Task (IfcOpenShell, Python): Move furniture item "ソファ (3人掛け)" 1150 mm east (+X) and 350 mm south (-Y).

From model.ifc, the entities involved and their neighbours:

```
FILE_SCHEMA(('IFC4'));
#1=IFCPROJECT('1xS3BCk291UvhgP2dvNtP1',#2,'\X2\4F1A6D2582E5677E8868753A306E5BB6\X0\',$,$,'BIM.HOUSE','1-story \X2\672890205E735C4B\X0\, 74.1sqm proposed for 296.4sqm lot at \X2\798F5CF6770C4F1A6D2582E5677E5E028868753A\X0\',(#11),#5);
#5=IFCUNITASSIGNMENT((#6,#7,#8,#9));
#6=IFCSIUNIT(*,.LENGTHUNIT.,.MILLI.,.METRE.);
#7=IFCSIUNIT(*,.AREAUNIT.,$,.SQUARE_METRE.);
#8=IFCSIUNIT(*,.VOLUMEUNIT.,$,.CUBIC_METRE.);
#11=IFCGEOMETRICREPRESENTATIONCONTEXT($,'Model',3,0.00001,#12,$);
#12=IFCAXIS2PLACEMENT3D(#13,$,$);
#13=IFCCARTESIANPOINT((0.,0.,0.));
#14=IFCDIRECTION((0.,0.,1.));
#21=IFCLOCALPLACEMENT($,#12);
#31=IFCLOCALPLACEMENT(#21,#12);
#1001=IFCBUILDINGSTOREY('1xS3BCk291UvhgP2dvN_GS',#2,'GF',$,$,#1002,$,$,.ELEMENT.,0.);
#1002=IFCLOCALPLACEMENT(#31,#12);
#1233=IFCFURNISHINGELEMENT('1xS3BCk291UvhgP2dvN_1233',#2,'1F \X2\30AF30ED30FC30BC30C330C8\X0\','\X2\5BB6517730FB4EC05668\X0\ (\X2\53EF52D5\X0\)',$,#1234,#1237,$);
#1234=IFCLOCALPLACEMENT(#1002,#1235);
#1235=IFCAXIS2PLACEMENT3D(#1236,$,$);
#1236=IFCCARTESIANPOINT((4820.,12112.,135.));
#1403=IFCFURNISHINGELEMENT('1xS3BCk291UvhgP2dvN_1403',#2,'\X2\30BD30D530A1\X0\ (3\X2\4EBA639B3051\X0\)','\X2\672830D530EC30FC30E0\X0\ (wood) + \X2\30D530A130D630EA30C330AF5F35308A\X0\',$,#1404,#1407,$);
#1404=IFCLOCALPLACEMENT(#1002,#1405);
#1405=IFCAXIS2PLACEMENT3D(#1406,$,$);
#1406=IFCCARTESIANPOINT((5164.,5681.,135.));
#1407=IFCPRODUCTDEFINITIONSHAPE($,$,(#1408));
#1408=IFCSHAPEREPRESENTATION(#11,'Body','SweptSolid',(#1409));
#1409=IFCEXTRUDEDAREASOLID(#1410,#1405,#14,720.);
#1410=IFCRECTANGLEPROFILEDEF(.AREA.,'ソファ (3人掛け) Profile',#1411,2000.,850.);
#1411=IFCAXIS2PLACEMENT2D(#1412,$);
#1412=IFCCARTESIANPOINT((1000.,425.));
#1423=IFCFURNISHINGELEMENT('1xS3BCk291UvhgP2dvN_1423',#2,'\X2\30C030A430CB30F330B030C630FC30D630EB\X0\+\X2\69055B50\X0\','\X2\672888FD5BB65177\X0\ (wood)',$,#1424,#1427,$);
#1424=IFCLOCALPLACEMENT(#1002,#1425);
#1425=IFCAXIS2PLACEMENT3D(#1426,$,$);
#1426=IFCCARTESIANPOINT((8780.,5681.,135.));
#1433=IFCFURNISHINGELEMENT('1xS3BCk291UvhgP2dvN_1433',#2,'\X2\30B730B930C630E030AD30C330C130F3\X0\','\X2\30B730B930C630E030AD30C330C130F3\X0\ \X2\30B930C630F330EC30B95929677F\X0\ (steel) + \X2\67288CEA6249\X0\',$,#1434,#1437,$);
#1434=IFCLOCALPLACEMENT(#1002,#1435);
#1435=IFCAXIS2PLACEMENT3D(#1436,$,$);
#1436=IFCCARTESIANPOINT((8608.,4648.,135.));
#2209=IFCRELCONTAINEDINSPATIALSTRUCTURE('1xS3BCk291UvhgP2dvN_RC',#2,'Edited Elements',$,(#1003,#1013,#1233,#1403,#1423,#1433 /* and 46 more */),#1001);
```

```python
import ifcopenshell
import ifcopenshell.api.geometry
import ifcopenshell.util.placement

model = ifcopenshell.open("model.ifc")

item = model.by_guid("1xS3BCk291UvhgP2dvN_1403")
matrix = ifcopenshell.util.placement.get_local_placement(item.ObjectPlacement)
matrix[0, 3] += 1150.0
matrix[1, 3] -= 350.0
ifcopenshell.api.geometry.edit_object_placement(model, product=item, matrix=matrix, is_si=False)

print(ifcopenshell.util.placement.get_local_placement(item.ObjectPlacement).round(3) + 0.0)

model.write("model-out.ifc")
```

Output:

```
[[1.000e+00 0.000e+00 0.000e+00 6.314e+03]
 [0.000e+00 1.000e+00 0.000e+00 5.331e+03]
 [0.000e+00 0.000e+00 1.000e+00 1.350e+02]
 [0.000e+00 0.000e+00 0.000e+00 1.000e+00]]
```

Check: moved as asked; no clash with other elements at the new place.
